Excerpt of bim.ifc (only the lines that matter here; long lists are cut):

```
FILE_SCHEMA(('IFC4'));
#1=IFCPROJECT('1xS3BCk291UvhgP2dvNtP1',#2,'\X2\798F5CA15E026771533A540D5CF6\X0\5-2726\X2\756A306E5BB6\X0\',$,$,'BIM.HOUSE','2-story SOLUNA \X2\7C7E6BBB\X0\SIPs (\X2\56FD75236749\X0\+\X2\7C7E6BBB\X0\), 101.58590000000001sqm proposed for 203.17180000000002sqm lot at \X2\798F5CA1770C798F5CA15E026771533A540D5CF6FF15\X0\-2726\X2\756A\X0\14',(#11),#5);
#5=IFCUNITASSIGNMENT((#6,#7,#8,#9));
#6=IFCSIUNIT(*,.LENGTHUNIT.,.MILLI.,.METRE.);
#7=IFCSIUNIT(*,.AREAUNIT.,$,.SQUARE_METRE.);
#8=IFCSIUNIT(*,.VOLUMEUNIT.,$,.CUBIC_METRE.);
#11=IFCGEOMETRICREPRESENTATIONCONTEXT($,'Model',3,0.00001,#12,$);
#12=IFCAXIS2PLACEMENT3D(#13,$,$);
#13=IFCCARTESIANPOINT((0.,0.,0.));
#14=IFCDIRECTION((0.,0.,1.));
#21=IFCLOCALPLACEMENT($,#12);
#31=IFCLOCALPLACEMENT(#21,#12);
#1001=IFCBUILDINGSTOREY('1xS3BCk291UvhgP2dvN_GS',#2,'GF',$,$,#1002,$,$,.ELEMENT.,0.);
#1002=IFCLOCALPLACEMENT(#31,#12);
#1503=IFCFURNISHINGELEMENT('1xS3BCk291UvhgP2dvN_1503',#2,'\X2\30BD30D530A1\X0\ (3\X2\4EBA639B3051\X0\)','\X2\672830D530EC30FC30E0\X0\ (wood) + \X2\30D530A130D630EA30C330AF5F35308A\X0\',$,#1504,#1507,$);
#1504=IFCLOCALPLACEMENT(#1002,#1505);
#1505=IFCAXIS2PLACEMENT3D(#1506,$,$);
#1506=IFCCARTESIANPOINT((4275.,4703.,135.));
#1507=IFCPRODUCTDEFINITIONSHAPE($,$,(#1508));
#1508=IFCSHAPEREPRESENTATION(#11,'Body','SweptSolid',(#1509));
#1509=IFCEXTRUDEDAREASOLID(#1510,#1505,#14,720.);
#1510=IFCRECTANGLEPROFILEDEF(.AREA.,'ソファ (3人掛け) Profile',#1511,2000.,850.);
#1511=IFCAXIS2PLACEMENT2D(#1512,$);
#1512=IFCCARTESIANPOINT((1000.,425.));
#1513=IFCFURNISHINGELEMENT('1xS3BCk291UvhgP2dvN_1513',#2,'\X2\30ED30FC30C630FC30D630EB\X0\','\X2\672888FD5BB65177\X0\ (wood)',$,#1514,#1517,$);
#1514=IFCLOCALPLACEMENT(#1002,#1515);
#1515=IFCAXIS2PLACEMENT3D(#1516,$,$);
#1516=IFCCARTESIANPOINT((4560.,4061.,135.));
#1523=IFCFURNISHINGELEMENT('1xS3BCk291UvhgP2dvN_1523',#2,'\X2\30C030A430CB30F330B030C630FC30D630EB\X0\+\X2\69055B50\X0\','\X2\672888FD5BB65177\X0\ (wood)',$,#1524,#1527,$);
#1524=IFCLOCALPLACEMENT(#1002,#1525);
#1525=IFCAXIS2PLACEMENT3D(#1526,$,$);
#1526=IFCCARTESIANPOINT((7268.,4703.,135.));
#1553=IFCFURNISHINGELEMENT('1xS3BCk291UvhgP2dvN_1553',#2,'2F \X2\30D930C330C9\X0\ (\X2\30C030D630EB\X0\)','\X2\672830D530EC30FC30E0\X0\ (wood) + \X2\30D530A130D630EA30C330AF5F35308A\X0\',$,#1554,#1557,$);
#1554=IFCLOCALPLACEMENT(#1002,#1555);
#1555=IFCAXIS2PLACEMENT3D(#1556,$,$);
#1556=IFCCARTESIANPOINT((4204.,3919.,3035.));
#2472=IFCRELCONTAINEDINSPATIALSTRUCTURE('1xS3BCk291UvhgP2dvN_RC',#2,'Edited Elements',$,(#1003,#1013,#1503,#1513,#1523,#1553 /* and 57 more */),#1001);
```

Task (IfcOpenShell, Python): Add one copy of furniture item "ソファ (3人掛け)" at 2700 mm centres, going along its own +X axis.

```python
import ifcopenshell
import ifcopenshell.api.geometry
import ifcopenshell.api.root
import ifcopenshell.util.element
import ifcopenshell.util.placement
import ifcopenshell.util.unit

model = ifcopenshell.open("bim.ifc")
unit_scale = ifcopenshell.util.unit.calculate_unit_scale(model)


def reuse_history(source, copy):
    """copy_class also copies each property set's owner history, people and application; keep the originals."""
    for rel in copy.IsDefinedBy:
        if rel.is_a("IfcRelDefinesByProperties") and (history := rel.RelatingPropertyDefinition.OwnerHistory):
            rel.RelatingPropertyDefinition.OwnerHistory = source.OwnerHistory
            ifcopenshell.util.element.remove_deep2(model, history)


source = model.by_guid("1xS3BCk291UvhgP2dvN_1503")
base = ifcopenshell.util.placement.get_local_placement(source.ObjectPlacement)
step = base[:3, 0] * 2.7 / unit_scale

for i in range(1, 2):
    copy = ifcopenshell.api.root.copy_class(model, product=source)
    copy.Representation = ifcopenshell.util.element.copy_deep(
        model, source.Representation, exclude=["IfcGeometricRepresentationContext", "IfcRepresentationMap"]
    )
    reuse_history(source, copy)
    matrix = base.copy()
    matrix[:3, 3] += i * step
    print("added at", matrix[:3, 3].round(3) + 0.0)
    ifcopenshell.api.geometry.edit_object_placement(model, product=copy, matrix=matrix, is_si=False)

model.write("bim_edited.ifc")
```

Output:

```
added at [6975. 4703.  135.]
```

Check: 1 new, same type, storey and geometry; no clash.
